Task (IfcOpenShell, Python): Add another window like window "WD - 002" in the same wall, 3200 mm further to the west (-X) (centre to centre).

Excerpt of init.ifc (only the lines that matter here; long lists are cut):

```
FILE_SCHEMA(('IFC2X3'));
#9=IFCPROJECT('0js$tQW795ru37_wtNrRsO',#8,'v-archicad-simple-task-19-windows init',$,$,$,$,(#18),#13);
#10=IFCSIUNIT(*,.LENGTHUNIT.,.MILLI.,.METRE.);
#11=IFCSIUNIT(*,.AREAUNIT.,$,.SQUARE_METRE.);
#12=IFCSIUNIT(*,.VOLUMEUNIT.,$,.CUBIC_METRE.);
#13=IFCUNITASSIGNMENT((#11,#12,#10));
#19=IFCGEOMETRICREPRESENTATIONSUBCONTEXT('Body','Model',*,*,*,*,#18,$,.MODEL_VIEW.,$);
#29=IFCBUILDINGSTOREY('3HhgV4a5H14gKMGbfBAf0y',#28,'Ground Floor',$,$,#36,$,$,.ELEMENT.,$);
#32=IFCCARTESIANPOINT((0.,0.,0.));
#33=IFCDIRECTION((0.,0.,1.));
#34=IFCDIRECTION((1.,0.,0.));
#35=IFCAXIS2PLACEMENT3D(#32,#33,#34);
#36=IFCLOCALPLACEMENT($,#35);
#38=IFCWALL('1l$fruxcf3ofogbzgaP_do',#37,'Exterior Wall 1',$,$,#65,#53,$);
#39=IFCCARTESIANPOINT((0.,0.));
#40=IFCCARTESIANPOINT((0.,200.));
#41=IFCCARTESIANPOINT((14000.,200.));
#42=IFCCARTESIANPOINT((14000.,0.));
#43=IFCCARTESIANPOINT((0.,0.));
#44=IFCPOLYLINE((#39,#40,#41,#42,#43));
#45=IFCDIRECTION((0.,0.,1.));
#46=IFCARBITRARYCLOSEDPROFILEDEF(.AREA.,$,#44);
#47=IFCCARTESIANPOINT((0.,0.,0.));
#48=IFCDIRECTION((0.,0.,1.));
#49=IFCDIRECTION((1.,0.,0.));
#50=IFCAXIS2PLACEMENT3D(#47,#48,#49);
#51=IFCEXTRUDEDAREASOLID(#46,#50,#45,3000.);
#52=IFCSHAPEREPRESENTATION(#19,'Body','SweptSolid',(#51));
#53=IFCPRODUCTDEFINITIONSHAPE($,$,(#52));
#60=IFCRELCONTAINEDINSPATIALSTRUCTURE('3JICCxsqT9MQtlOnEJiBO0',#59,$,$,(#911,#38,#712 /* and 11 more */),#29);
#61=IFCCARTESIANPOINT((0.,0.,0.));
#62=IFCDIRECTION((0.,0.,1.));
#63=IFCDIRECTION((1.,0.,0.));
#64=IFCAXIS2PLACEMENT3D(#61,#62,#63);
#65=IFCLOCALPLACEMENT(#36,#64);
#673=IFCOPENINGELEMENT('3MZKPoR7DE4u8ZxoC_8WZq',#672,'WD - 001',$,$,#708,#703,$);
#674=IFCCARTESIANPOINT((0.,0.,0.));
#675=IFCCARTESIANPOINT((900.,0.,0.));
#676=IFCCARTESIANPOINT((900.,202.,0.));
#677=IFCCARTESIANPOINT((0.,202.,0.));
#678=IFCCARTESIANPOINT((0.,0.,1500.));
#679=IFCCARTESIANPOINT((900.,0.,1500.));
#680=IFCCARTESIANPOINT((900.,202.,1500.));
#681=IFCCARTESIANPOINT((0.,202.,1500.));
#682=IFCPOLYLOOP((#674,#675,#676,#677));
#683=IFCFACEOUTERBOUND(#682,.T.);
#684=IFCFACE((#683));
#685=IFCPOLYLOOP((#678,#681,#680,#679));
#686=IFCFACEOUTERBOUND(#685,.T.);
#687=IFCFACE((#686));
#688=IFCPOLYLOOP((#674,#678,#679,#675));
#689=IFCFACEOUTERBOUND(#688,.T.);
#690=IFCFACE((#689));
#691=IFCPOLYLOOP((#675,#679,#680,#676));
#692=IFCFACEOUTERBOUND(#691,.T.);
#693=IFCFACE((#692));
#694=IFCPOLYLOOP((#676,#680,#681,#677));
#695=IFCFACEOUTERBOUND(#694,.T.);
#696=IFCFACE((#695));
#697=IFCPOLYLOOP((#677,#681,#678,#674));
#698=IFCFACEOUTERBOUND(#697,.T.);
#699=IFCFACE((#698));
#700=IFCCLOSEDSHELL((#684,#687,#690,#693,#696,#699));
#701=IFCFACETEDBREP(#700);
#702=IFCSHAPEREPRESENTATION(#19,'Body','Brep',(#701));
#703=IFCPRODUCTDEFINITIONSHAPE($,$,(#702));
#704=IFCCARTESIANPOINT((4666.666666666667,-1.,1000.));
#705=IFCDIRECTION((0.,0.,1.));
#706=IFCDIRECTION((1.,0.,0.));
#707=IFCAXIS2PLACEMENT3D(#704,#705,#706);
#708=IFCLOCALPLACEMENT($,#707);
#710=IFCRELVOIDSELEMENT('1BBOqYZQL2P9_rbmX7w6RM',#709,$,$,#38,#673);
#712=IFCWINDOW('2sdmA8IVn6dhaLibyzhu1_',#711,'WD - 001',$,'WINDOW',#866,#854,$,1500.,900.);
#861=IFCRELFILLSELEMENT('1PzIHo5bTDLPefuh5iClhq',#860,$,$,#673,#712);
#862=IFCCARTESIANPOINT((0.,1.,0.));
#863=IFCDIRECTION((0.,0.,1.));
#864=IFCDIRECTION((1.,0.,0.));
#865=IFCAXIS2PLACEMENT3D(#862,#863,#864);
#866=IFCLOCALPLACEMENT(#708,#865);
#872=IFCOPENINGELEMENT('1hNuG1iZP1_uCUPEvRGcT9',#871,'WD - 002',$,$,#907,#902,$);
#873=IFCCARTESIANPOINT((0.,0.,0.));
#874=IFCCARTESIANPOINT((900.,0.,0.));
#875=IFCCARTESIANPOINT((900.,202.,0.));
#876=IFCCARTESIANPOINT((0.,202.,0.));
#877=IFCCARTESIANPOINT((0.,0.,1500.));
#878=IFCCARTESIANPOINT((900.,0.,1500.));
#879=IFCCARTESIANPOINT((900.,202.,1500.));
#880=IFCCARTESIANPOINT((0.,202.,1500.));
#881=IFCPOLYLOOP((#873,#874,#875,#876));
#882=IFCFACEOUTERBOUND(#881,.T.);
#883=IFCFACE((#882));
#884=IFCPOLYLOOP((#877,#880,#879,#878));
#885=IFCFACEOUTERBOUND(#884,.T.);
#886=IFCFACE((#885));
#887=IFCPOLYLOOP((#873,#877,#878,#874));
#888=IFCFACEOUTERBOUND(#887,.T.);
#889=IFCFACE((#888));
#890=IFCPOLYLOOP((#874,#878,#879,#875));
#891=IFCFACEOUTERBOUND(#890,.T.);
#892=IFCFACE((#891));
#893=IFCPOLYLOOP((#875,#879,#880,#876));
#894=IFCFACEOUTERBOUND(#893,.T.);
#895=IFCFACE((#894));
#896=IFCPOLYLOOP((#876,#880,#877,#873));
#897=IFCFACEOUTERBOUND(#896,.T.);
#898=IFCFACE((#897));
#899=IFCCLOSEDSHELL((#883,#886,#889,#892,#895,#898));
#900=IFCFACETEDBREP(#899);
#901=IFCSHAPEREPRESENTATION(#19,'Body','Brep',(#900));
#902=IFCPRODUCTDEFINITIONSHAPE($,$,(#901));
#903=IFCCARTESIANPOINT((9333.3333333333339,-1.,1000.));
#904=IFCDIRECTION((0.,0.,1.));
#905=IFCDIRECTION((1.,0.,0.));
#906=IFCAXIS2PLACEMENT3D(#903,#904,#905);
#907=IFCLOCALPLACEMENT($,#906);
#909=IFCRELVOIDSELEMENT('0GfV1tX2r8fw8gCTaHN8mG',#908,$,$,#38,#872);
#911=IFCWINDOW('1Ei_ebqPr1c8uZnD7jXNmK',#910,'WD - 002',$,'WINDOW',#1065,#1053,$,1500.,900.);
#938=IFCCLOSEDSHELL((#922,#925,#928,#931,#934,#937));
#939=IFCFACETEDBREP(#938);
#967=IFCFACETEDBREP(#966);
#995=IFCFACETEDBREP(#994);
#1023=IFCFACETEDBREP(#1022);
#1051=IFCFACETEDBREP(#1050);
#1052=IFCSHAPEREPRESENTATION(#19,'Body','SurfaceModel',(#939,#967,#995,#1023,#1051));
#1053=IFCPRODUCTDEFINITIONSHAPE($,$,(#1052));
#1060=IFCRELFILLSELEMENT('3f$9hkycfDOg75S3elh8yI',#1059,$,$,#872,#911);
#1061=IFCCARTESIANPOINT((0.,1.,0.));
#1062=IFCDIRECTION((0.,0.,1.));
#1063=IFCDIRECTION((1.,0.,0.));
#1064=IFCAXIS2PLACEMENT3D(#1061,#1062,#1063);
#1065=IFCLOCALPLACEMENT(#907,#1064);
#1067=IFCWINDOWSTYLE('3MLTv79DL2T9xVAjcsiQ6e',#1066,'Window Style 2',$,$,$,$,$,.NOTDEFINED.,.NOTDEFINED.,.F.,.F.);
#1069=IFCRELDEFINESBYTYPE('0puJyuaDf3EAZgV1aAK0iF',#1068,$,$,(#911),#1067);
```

```python
import ifcopenshell
import ifcopenshell.api.feature
import ifcopenshell.api.geometry
import ifcopenshell.api.root
import ifcopenshell.geom
import ifcopenshell.util.element
import ifcopenshell.util.placement
import ifcopenshell.util.shape
import ifcopenshell.util.unit

model = ifcopenshell.open("init.ifc")
unit_scale = ifcopenshell.util.unit.calculate_unit_scale(model)
settings = ifcopenshell.geom.settings()


def volume(element):
    """Net volume in cubic metres, openings subtracted."""
    shape = ifcopenshell.geom.create_shape(settings, element)
    return ifcopenshell.util.shape.get_volume(shape.geometry)


window = model.by_guid("1Ei_ebqPr1c8uZnD7jXNmK")
opening = window.FillsVoids[0].RelatingOpeningElement
wall = opening.VoidsElements[0].RelatingBuildingElement
before = volume(wall)
shift = ifcopenshell.util.placement.get_local_placement(wall.ObjectPlacement)[:3, 0] * -3.2 / unit_scale

# copy_class copies the void relationship, type, container and properties, but no geometry.
new_opening = ifcopenshell.api.root.copy_class(model, product=opening)
new_opening.Representation = ifcopenshell.util.element.copy_deep(
    model, opening.Representation, exclude=["IfcGeometricRepresentationContext", "IfcRepresentationMap"]
)
new_window = ifcopenshell.api.root.copy_class(model, product=window)
new_window.Representation = ifcopenshell.util.element.copy_deep(
    model, window.Representation, exclude=["IfcGeometricRepresentationContext", "IfcRepresentationMap"]
)
fills = ifcopenshell.api.feature.add_filling(model, opening=new_opening, element=new_window)
fills.OwnerHistory = new_window.OwnerHistory  # required in IFC2X3

for old, new in ((opening, new_opening), (window, new_window)):
    matrix = ifcopenshell.util.placement.get_local_placement(old.ObjectPlacement)
    matrix[:3, 3] += shift
    ifcopenshell.api.geometry.edit_object_placement(model, product=new, matrix=matrix, is_si=False)

after = volume(wall)

print(f"wall volume {before:.3f} -> {after:.3f} m3")

model.write("init_updated.ifc")
```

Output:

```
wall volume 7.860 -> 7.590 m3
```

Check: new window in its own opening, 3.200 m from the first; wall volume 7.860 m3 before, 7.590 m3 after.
